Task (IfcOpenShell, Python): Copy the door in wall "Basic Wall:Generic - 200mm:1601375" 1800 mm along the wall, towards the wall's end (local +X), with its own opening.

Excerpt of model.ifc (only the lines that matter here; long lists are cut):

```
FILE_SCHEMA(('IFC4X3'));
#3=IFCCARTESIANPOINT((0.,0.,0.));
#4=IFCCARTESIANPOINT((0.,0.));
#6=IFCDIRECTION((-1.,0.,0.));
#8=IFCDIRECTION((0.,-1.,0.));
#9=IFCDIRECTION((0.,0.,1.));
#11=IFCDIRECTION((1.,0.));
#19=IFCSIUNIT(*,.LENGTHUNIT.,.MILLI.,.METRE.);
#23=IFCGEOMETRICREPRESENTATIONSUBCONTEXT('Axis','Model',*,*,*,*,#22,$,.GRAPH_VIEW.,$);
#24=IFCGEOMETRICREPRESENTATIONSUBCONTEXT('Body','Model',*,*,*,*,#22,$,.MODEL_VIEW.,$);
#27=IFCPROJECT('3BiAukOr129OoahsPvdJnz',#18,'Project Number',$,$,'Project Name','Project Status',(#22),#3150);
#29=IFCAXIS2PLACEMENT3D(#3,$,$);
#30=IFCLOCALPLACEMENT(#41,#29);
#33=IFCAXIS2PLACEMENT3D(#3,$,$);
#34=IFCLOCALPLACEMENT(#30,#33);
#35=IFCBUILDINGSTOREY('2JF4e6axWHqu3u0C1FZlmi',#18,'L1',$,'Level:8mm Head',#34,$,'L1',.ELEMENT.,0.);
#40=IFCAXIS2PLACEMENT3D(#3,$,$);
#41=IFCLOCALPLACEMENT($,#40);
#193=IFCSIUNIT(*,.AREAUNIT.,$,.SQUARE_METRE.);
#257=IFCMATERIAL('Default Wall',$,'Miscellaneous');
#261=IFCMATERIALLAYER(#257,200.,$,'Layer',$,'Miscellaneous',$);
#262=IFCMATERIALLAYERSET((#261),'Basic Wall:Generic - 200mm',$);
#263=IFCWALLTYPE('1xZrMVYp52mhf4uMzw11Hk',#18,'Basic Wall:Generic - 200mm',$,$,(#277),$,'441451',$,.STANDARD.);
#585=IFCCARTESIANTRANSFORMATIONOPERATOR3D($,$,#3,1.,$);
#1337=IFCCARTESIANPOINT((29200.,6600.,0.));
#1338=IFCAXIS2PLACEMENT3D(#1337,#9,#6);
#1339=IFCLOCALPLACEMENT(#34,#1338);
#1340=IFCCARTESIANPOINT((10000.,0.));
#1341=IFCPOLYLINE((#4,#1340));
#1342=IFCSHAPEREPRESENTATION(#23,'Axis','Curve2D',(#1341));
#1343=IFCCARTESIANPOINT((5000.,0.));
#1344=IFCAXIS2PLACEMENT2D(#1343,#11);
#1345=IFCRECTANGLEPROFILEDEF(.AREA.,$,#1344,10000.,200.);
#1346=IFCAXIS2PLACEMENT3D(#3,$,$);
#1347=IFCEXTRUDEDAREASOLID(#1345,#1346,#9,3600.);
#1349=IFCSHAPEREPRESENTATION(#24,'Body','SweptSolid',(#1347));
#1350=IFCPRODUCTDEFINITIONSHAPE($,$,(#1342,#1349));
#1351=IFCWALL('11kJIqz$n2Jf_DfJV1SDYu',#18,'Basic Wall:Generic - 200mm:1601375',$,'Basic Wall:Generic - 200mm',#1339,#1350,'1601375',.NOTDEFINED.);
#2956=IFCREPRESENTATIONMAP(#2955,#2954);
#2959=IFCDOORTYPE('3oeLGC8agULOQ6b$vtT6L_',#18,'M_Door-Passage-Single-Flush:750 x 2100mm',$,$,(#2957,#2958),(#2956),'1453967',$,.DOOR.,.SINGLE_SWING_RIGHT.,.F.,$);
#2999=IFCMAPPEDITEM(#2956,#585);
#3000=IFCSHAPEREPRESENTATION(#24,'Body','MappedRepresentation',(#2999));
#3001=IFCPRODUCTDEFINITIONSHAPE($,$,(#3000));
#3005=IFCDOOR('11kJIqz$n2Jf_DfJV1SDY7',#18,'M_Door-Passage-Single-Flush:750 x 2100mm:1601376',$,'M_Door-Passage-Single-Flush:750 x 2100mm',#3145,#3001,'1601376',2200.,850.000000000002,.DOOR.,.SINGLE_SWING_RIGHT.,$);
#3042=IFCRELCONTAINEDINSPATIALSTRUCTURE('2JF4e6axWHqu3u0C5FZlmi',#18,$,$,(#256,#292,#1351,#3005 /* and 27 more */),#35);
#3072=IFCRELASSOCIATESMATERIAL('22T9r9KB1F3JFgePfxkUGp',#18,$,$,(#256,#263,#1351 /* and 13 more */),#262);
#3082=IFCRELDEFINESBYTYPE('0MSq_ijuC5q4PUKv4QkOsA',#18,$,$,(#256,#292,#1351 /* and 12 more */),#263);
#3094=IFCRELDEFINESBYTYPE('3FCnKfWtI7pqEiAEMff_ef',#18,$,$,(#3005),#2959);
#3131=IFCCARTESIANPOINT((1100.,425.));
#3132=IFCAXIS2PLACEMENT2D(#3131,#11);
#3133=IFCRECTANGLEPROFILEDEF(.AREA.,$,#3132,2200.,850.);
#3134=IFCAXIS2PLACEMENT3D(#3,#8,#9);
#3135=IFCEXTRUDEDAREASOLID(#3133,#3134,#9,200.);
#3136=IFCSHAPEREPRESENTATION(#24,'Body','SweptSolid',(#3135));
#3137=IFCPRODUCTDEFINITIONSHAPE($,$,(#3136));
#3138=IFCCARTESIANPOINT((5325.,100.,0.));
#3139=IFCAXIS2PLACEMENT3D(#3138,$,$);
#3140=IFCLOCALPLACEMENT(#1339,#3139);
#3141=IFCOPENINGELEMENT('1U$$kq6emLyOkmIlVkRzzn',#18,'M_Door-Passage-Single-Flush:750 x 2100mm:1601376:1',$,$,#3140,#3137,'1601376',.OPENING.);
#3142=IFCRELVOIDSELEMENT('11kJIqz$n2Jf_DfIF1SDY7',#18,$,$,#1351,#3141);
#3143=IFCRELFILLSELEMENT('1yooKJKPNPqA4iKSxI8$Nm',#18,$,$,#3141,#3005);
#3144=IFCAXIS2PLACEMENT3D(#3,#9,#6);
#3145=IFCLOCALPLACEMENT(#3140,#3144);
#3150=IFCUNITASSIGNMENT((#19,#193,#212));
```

```python
import ifcopenshell
import ifcopenshell.api.feature
import ifcopenshell.api.geometry
import ifcopenshell.api.root
import ifcopenshell.geom
import ifcopenshell.util.element
import ifcopenshell.util.placement
import ifcopenshell.util.shape

model = ifcopenshell.open("model.ifc")
settings = ifcopenshell.geom.settings()


def volume(element):
    """Net volume in cubic metres, openings subtracted."""
    shape = ifcopenshell.geom.create_shape(settings, element)
    return ifcopenshell.util.shape.get_volume(shape.geometry)


def reuse_history(source, copy):
    """copy_class also copies each property set's owner history, people and application; keep the originals."""
    for rel in copy.IsDefinedBy:
        if rel.is_a("IfcRelDefinesByProperties") and (history := rel.RelatingPropertyDefinition.OwnerHistory):
            rel.RelatingPropertyDefinition.OwnerHistory = source.OwnerHistory
            ifcopenshell.util.element.remove_deep2(model, history)


door = model.by_guid("11kJIqz$n2Jf_DfJV1SDY7")
opening = door.FillsVoids[0].RelatingOpeningElement
wall = opening.VoidsElements[0].RelatingBuildingElement
before = volume(wall)
shift = ifcopenshell.util.placement.get_local_placement(wall.ObjectPlacement)[:3, 0] * 1800.0

# copy_class copies the void relationship, type, container and properties, but no geometry.
new_opening = ifcopenshell.api.root.copy_class(model, product=opening)
new_opening.Representation = ifcopenshell.util.element.copy_deep(
    model, opening.Representation, exclude=["IfcGeometricRepresentationContext", "IfcRepresentationMap"]
)
new_opening.Name = "M_Door-Passage-Single-Flush:750 x 2100mm"
new_opening.Tag = None
new_door = ifcopenshell.api.root.copy_class(model, product=door)
new_door.Representation = ifcopenshell.util.element.copy_deep(
    model, door.Representation, exclude=["IfcGeometricRepresentationContext", "IfcRepresentationMap"]
)
new_door.Name = "M_Door-Passage-Single-Flush:750 x 2100mm"
new_door.Tag = None
reuse_history(door, new_door)
ifcopenshell.api.feature.add_filling(model, opening=new_opening, element=new_door)

for old, new in ((opening, new_opening), (door, new_door)):
    matrix = ifcopenshell.util.placement.get_local_placement(old.ObjectPlacement)
    matrix[:3, 3] += shift
    ifcopenshell.api.geometry.edit_object_placement(model, product=new, matrix=matrix, is_si=False)

after = volume(wall)

print(f"wall volume {before:.3f} -> {after:.3f} m3")

model.write("model_v2.ifc")
```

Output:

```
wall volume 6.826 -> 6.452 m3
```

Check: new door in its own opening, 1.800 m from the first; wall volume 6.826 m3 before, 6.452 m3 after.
